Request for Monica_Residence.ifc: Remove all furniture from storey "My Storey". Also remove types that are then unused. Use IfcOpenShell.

First a look at what the model holds.

```python
import ifcopenshell
import ifcopenshell.util.element

model = ifcopenshell.open("Monica_Residence.ifc")
print(model.schema)
storey = next(s for s in model.by_type("IfcBuildingStorey") if s.Name == "My Storey")
furniture = [e for e in ifcopenshell.util.element.get_decomposition(storey) if e.is_a("IfcFurnishingElement")]
seen = {}
for e in furniture:
    element_type = ifcopenshell.util.element.get_type(e)
    name = element_type.Name if element_type not in (None, e) else None
    seen[name] = seen.get(name, 0) + 1
for name, count in sorted(seen.items(), key=str):
    print(count, "x", name)
```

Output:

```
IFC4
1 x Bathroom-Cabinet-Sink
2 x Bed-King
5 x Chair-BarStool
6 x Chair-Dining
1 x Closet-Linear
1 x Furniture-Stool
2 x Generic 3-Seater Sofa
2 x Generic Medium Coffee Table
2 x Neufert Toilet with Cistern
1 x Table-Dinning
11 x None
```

```python
import ifcopenshell
import ifcopenshell.api.root
import ifcopenshell.util.element

model = ifcopenshell.open("Monica_Residence.ifc")

storey = next(s for s in model.by_type("IfcBuildingStorey") if s.Name == "My Storey")
furniture = [e for e in ifcopenshell.util.element.get_decomposition(storey) if e.is_a("IfcFurnishingElement")]
types = {ifcopenshell.util.element.get_type(e) for e in furniture} - {None, *furniture}

for e in furniture:
    ifcopenshell.api.root.remove_product(model, product=e)
print(len(furniture), "removed")

unused = [t for t in types if not ifcopenshell.util.element.get_types(t)]
for t in unused:
    ifcopenshell.api.root.remove_product(model, product=t)
print(len(unused), "unused types removed")

model.write("Monica_Residence_updated.ifc")
```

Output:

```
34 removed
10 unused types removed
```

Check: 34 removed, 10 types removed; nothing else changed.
